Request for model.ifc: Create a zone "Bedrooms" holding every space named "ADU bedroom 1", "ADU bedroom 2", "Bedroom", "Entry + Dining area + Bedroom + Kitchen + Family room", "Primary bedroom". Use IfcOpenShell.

First a look at what the model holds.

```python
import ifcopenshell

model = ifcopenshell.open("model.ifc")
print(model.schema)
seen = {}
for space in model.by_type("IfcSpace"):
    seen[space.Name] = seen.get(space.Name, 0) + 1
for name, count in sorted(seen.items(), key=str):
    print(count, "x", name)
print("zones:", [z.Name for z in model.by_type("IfcZone")][:20])
```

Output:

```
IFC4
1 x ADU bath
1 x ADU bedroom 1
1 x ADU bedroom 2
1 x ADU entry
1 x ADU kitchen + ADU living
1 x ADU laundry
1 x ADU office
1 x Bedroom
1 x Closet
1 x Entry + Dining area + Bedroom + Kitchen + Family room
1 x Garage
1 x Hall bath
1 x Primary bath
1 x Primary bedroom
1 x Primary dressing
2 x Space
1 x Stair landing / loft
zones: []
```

```python
import ifcopenshell
import ifcopenshell.api.group
import ifcopenshell.api.root

model = ifcopenshell.open("model.ifc")

names = {"ADU bedroom 1", "ADU bedroom 2", "Bedroom", "Entry + Dining area + Bedroom + Kitchen + Family room", "Primary bedroom"}
spaces = [s for s in model.by_type("IfcSpace") if s.Name in names]

zone = ifcopenshell.api.root.create_entity(model, ifc_class="IfcZone", name="Bedrooms")
ifcopenshell.api.group.assign_group(model, products=spaces, group=zone)
print(len(spaces), "spaces in", zone.Name)

model.write("model_updated.ifc")
```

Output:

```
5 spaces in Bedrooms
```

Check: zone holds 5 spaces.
